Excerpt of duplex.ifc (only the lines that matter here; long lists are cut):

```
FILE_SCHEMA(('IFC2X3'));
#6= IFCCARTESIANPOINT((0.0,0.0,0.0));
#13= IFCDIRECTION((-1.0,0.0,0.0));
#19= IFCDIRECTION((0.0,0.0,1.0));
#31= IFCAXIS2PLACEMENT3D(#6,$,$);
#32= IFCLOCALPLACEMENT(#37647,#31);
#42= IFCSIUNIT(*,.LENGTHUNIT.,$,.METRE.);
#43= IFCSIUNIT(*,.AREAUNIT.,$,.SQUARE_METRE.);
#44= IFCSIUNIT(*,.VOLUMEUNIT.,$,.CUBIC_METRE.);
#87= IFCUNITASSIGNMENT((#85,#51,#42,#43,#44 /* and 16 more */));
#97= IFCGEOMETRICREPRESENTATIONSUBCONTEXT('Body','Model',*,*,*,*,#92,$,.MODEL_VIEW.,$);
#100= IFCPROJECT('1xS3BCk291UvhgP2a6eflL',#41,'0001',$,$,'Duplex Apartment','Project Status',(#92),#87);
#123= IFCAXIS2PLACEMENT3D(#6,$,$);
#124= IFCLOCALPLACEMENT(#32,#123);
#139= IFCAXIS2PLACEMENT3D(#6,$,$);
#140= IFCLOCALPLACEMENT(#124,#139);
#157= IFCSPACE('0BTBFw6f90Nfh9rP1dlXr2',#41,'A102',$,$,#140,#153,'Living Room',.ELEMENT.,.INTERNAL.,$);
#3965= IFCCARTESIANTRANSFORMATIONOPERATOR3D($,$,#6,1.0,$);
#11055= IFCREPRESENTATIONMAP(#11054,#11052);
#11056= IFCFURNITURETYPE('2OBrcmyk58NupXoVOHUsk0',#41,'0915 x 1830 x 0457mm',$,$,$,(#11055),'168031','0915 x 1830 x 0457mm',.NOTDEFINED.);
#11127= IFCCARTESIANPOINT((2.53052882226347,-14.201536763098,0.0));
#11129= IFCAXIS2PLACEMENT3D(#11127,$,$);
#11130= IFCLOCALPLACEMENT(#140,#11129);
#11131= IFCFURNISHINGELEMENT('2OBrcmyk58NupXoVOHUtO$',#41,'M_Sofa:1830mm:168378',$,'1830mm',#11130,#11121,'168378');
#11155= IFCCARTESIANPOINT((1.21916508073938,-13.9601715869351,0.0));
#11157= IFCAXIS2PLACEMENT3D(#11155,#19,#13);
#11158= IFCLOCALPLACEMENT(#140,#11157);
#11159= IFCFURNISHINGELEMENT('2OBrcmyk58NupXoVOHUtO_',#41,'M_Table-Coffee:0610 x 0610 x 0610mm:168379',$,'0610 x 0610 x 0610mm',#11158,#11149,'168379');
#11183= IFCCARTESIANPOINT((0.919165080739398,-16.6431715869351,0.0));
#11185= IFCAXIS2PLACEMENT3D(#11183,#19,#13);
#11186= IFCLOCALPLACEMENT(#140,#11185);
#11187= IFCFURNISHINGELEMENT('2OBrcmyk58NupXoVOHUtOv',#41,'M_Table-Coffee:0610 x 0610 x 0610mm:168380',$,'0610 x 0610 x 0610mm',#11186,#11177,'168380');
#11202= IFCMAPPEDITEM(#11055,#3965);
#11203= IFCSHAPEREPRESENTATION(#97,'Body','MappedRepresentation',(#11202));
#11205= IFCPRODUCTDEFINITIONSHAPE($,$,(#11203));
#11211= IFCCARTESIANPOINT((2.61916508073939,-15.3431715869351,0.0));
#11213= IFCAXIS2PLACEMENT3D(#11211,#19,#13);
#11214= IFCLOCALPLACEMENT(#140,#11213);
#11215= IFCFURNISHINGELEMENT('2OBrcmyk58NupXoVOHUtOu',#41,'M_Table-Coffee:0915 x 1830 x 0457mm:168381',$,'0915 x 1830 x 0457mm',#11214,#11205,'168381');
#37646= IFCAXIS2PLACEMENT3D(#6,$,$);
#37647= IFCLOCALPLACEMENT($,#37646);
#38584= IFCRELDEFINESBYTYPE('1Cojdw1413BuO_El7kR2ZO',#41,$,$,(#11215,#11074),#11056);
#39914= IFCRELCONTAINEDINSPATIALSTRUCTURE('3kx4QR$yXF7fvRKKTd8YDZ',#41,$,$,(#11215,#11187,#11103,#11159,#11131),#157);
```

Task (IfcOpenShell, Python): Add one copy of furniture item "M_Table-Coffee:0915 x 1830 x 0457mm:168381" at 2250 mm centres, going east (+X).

```python
import numpy as np
import ifcopenshell
import ifcopenshell.api.geometry
import ifcopenshell.api.root
import ifcopenshell.util.element
import ifcopenshell.util.placement
import ifcopenshell.util.unit

model = ifcopenshell.open("duplex.ifc")
unit_scale = ifcopenshell.util.unit.calculate_unit_scale(model)


def reuse_history(source, copy):
    """copy_class also copies each property set's owner history, people and application; keep the originals."""
    for rel in copy.IsDefinedBy:
        if rel.is_a("IfcRelDefinesByProperties") and (history := rel.RelatingPropertyDefinition.OwnerHistory):
            rel.RelatingPropertyDefinition.OwnerHistory = source.OwnerHistory
            ifcopenshell.util.element.remove_deep2(model, history)


source = model.by_guid("2OBrcmyk58NupXoVOHUtOu")
base = ifcopenshell.util.placement.get_local_placement(source.ObjectPlacement)
step = np.array([1.0, 0.0, 0.0]) * 2.25 / unit_scale

for i in range(1, 2):
    copy = ifcopenshell.api.root.copy_class(model, product=source)
    copy.Representation = ifcopenshell.util.element.copy_deep(
        model, source.Representation, exclude=["IfcGeometricRepresentationContext", "IfcRepresentationMap"]
    )
    copy.Name = "M_Table-Coffee:0915 x 1830 x 0457mm"
    copy.Tag = None
    reuse_history(source, copy)
    matrix = base.copy()
    matrix[:3, 3] += i * step
    print("added at", matrix[:3, 3].round(3) + 0.0)
    ifcopenshell.api.geometry.edit_object_placement(model, product=copy, matrix=matrix, is_si=False)

model.write("duplex_rev.ifc")
```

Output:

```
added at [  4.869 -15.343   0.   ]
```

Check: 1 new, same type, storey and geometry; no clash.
